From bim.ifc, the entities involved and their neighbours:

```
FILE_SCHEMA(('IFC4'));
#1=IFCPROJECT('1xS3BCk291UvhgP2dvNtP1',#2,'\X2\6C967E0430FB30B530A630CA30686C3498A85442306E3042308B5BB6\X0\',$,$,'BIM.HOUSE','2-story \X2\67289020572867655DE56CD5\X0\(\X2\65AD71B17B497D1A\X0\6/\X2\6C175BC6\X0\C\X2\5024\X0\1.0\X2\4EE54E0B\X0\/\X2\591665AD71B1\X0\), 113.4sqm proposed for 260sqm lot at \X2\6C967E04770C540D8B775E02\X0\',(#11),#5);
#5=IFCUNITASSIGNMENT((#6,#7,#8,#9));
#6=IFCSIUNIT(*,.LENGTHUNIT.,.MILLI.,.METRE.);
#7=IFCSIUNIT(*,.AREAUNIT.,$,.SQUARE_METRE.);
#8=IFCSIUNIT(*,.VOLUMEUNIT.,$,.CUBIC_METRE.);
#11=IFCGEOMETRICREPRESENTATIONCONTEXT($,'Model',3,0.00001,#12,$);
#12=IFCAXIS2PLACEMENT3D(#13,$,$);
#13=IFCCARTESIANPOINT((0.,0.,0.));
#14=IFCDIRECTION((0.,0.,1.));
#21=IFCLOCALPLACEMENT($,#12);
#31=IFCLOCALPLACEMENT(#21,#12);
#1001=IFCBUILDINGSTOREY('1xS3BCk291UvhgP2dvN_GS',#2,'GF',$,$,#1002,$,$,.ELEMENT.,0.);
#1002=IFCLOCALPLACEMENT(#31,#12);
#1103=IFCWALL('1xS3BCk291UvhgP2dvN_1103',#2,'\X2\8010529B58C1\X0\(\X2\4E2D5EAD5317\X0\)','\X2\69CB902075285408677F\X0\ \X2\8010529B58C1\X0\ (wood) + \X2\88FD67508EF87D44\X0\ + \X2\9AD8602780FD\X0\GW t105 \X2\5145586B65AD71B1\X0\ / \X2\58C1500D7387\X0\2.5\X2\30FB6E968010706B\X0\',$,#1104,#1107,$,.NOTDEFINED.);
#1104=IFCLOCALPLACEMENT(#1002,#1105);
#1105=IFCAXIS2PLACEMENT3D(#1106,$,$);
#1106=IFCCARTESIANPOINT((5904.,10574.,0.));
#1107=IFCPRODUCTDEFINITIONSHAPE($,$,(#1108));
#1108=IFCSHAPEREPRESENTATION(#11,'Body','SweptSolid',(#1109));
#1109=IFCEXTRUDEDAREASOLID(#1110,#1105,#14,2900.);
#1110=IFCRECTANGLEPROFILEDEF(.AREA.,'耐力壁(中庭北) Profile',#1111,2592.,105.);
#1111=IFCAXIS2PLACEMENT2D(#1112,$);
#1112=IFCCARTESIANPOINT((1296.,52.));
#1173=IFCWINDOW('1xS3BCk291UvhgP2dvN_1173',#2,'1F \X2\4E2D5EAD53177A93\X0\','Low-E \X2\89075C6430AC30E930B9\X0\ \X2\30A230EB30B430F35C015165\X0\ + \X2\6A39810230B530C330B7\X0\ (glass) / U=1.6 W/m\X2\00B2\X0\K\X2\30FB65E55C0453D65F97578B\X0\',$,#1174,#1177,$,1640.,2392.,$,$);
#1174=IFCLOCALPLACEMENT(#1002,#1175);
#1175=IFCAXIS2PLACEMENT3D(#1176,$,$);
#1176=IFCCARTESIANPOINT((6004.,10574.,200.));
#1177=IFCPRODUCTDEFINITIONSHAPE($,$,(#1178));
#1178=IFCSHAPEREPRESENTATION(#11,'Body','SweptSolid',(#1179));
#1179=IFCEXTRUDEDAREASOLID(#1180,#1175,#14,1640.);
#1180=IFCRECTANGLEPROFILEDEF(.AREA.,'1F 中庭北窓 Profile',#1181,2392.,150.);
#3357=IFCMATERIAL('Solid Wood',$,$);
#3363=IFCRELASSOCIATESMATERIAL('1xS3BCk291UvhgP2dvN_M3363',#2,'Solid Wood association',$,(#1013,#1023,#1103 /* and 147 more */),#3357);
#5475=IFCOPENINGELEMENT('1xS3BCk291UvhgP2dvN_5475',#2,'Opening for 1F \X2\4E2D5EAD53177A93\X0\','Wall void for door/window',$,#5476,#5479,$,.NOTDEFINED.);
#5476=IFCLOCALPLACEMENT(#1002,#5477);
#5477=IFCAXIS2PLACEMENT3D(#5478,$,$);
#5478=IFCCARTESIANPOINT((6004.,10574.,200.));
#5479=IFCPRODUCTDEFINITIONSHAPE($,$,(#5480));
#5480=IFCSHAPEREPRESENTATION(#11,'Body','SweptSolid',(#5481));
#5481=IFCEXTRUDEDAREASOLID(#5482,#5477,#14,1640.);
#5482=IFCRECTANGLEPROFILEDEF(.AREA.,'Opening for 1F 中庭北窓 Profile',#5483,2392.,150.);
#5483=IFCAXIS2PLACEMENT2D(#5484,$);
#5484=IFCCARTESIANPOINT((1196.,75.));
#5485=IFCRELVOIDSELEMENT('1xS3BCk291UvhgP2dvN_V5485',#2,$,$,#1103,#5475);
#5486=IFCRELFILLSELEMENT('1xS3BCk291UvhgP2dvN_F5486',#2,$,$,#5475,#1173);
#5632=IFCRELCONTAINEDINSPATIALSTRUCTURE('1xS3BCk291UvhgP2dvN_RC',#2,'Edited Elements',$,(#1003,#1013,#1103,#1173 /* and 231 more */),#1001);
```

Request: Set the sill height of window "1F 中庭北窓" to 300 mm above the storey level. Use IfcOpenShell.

```python
import numpy as np
import ifcopenshell
import ifcopenshell.api.geometry
import ifcopenshell.geom
import ifcopenshell.util.element
import ifcopenshell.util.placement
import ifcopenshell.util.shape
import ifcopenshell.util.unit

model = ifcopenshell.open("bim.ifc")
unit_scale = ifcopenshell.util.unit.calculate_unit_scale(model)

window = model.by_id(1173)
opening = window.FillsVoids[0].RelatingOpeningElement
storey = ifcopenshell.util.element.get_container(window, ifc_class="IfcBuildingStorey")
level = ifcopenshell.util.placement.get_local_placement(storey.ObjectPlacement)[2, 3]

# The opening's origin need not be at the sill, so measure its lowest point.
shape = ifcopenshell.geom.create_shape(ifcopenshell.geom.settings(), opening)
bottom = ifcopenshell.util.shape.get_shape_bottom_elevation(shape, shape.geometry) / unit_scale
dz = level + 0.3 / unit_scale - bottom

shift = np.array([0.0, 0.0, dz])
# The window is not placed relative to its opening, so move both.
for product in (opening, window):
    matrix = ifcopenshell.util.placement.get_local_placement(product.ObjectPlacement)
    matrix[:3, 3] += shift
    ifcopenshell.api.geometry.edit_object_placement(model, product=product, matrix=matrix, is_si=False)

print(f"moved by {dz * unit_scale:+.3f} m")

model.write("bim_rev.ifc")
```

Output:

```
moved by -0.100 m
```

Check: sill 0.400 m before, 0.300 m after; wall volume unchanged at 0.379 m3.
